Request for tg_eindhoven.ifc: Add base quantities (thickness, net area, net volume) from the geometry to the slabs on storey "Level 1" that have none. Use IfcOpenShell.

First a look at what the model holds.

```python
import ifcopenshell
import ifcopenshell.util.element
import ifcopenshell.util.unit

model = ifcopenshell.open("tg_eindhoven.ifc")
print(model.schema)
for unit_type in ("LENGTHUNIT", "AREAUNIT", "VOLUMEUNIT"):
    print(unit_type, ifcopenshell.util.unit.calculate_unit_scale(model, unit_type))
storey = next(s for s in model.by_type("IfcBuildingStorey") if s.Name == "Level 1")
slabs = [e for e in ifcopenshell.util.element.get_decomposition(storey) if e.is_a("IfcSlab")]
for e in sorted(slabs, key=lambda e: e.id()):
    print(e.id(), e.is_a(), e.Name, list(ifcopenshell.util.element.get_psets(e, qtos_only=True)), sep=" | ")
```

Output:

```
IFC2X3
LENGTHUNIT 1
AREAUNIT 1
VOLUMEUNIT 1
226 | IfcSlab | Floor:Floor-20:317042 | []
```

```python
import ifcopenshell
import ifcopenshell.api.pset
import ifcopenshell.geom
import ifcopenshell.util.element
import ifcopenshell.util.shape
import ifcopenshell.util.unit

model = ifcopenshell.open("tg_eindhoven.ifc")
unit_scale = ifcopenshell.util.unit.calculate_unit_scale(model)
area_scale = ifcopenshell.util.unit.calculate_unit_scale(model, "AREAUNIT")
volume_scale = ifcopenshell.util.unit.calculate_unit_scale(model, "VOLUMEUNIT")
settings = ifcopenshell.geom.settings()

storey = next(s for s in model.by_type("IfcBuildingStorey") if s.Name == "Level 1")
slabs = [e for e in ifcopenshell.util.element.get_decomposition(storey) if e.is_a("IfcSlab")]

for e in sorted(slabs, key=lambda e: e.id()):
    if ifcopenshell.util.element.get_psets(e, qtos_only=True, should_inherit=False):
        continue
    # Geometry comes back in metres, in the element's own axes.
    shape = ifcopenshell.geom.create_shape(settings, e)
    values = {
        "Width": ifcopenshell.util.shape.get_z(shape.geometry) / unit_scale,
        "NetArea": ifcopenshell.util.shape.get_footprint_area(shape.geometry) / area_scale,
        "NetVolume": ifcopenshell.util.shape.get_volume(shape.geometry) / volume_scale,
    }
    qto = ifcopenshell.api.pset.add_qto(model, product=e, name="BaseQuantities")
    ifcopenshell.api.pset.edit_qto(model, qto=qto, properties=values)
    print(e.id(), {k: round(v, 3) for k, v in values.items()})

model.write("tg_eindhoven_updated.ifc")
```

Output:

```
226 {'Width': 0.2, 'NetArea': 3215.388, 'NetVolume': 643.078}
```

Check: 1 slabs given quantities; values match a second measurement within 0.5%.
